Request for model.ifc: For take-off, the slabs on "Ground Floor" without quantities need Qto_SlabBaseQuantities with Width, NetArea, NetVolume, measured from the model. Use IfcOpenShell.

First a look at what the model holds.

```python
import ifcopenshell
import ifcopenshell.util.element
import ifcopenshell.util.unit

model = ifcopenshell.open("model.ifc")
print(model.schema)
for unit_type in ("LENGTHUNIT", "AREAUNIT", "VOLUMEUNIT"):
    print(unit_type, ifcopenshell.util.unit.calculate_unit_scale(model, unit_type))
storey = next(s for s in model.by_type("IfcBuildingStorey") if s.Name == "Ground Floor")
slabs = [e for e in ifcopenshell.util.element.get_decomposition(storey) if e.is_a("IfcSlab")]
for e in sorted(slabs, key=lambda e: e.id()):
    print(e.id(), e.is_a(), e.Name, list(ifcopenshell.util.element.get_psets(e, qtos_only=True)), sep=" | ")
```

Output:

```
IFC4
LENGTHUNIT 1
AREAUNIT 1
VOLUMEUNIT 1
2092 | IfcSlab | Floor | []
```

```python
import ifcopenshell
import ifcopenshell.api.pset
import ifcopenshell.geom
import ifcopenshell.util.element
import ifcopenshell.util.shape
import ifcopenshell.util.unit

model = ifcopenshell.open("model.ifc")
unit_scale = ifcopenshell.util.unit.calculate_unit_scale(model)
area_scale = ifcopenshell.util.unit.calculate_unit_scale(model, "AREAUNIT")
volume_scale = ifcopenshell.util.unit.calculate_unit_scale(model, "VOLUMEUNIT")
settings = ifcopenshell.geom.settings()

storey = next(s for s in model.by_type("IfcBuildingStorey") if s.Name == "Ground Floor")
slabs = [e for e in ifcopenshell.util.element.get_decomposition(storey) if e.is_a("IfcSlab")]

for e in sorted(slabs, key=lambda e: e.id()):
    if ifcopenshell.util.element.get_psets(e, qtos_only=True, should_inherit=False):
        continue
    # Geometry comes back in metres, in the element's own axes.
    shape = ifcopenshell.geom.create_shape(settings, e)
    values = {
        "Width": ifcopenshell.util.shape.get_z(shape.geometry) / unit_scale,
        "NetArea": ifcopenshell.util.shape.get_footprint_area(shape.geometry) / area_scale,
        "NetVolume": ifcopenshell.util.shape.get_volume(shape.geometry) / volume_scale,
    }
    qto = ifcopenshell.api.pset.add_qto(model, product=e, name="Qto_SlabBaseQuantities")
    ifcopenshell.api.pset.edit_qto(model, qto=qto, properties=values)
    print(e.id(), {k: round(v, 3) for k, v in values.items()})

model.write("model_rev.ifc")
```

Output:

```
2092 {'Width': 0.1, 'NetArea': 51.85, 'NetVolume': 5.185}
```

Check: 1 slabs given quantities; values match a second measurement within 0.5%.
